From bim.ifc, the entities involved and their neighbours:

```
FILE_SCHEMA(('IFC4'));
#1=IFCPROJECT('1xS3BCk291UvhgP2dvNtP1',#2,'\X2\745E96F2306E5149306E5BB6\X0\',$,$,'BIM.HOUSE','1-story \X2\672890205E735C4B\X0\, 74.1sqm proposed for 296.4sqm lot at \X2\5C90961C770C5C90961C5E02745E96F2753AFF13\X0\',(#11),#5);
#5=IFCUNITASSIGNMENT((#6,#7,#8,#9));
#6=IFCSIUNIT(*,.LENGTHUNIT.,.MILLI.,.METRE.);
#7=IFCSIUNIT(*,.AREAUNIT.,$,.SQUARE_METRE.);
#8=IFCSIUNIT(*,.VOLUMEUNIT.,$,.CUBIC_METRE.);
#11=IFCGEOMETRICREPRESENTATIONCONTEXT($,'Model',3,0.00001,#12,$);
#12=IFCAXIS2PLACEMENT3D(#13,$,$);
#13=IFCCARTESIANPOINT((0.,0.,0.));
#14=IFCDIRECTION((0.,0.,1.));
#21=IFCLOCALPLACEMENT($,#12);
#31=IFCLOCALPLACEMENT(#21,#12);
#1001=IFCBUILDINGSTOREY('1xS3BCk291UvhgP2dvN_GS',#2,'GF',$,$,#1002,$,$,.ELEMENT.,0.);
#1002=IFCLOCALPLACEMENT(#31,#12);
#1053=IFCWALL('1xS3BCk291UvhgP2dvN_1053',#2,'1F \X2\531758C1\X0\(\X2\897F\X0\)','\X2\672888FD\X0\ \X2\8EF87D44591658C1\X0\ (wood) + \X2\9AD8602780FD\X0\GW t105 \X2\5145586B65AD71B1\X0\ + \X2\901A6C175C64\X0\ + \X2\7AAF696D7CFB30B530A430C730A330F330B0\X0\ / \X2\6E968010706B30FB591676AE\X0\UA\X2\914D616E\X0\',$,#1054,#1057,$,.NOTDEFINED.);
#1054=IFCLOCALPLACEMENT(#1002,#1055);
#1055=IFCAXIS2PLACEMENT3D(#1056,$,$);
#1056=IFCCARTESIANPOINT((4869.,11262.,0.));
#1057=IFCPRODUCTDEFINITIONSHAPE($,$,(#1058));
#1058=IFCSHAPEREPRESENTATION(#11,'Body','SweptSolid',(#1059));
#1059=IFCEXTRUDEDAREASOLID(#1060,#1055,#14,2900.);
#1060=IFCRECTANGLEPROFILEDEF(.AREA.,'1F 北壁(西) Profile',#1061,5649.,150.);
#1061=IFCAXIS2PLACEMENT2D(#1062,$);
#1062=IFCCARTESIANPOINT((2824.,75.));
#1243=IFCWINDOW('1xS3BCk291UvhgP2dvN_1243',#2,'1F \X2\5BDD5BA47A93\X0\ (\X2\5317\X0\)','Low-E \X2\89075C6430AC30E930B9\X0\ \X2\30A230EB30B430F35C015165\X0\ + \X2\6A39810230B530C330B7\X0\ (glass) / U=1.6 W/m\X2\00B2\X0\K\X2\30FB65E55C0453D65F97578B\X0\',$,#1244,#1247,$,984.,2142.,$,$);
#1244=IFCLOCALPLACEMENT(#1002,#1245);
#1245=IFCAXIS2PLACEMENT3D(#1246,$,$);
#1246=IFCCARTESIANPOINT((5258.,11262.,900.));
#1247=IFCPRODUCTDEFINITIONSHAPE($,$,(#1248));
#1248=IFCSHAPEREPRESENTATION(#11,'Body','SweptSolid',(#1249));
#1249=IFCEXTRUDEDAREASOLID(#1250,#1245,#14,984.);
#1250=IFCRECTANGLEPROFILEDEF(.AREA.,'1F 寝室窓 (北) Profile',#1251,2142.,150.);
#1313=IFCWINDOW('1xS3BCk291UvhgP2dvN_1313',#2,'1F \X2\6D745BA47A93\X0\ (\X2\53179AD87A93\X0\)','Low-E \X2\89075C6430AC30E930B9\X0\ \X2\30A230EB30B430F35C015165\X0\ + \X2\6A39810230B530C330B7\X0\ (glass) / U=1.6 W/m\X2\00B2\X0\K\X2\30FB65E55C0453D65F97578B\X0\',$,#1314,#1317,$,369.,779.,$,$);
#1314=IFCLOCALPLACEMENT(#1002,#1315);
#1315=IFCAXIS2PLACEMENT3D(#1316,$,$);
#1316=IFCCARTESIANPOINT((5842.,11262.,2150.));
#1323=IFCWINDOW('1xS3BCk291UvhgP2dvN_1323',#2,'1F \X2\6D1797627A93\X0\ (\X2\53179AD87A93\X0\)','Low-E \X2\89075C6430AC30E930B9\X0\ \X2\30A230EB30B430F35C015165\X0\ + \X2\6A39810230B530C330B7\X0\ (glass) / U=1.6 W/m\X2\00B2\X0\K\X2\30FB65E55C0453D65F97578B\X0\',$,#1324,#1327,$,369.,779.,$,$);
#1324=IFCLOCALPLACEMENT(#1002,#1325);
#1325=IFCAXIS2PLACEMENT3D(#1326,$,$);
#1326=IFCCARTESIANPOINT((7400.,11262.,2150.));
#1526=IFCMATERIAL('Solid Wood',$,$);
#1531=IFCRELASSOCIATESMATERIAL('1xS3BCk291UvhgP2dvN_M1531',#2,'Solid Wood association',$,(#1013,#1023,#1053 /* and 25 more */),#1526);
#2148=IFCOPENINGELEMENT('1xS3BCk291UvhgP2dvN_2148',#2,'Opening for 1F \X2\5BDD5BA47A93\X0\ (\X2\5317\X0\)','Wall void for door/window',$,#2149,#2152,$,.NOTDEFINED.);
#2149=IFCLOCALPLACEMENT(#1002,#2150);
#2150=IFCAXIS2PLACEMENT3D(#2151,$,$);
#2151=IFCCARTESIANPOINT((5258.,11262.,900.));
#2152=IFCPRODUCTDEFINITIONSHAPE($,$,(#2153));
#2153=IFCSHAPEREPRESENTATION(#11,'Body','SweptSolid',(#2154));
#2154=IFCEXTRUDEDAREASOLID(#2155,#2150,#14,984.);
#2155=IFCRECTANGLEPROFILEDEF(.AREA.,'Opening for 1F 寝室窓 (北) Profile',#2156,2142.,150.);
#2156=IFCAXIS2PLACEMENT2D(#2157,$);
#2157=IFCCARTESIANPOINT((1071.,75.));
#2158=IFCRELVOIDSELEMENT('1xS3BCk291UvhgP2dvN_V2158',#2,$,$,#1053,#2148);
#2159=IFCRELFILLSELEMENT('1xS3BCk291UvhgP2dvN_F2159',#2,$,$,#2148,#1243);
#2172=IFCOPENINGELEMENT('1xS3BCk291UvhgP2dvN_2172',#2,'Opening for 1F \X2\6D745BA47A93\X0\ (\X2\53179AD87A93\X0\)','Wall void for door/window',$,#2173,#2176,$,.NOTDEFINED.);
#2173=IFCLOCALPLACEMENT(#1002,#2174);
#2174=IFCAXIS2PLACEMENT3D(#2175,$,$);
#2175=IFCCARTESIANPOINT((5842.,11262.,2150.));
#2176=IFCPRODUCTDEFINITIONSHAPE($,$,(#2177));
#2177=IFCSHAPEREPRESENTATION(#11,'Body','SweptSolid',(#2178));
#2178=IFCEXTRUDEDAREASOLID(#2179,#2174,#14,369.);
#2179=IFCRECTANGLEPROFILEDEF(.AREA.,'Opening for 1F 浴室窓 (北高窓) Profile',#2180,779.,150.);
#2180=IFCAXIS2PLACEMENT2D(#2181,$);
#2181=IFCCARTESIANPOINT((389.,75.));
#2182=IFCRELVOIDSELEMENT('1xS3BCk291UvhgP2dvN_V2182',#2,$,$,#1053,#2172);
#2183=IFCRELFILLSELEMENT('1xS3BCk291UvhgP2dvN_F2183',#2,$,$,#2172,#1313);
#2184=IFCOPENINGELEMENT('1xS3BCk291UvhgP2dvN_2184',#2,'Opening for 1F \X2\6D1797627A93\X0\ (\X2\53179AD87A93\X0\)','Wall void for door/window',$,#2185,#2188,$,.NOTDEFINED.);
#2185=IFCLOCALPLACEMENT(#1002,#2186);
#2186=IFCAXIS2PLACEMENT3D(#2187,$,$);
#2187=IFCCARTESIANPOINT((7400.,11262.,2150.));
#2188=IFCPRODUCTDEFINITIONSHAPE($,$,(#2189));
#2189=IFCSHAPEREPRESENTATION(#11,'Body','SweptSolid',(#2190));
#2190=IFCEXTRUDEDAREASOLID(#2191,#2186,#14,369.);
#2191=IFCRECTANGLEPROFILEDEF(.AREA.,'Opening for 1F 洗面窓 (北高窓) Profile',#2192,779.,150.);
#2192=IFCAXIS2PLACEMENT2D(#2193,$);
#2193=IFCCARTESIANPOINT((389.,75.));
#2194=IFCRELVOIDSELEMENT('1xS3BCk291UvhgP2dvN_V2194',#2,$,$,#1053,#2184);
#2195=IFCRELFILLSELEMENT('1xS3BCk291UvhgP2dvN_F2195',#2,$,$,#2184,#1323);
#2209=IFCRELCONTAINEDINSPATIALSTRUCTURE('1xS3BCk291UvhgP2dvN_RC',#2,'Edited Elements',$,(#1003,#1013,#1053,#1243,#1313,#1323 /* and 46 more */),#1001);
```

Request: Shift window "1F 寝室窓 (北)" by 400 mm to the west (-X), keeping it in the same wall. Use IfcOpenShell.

```python
import ifcopenshell
import ifcopenshell.api.geometry
import ifcopenshell.util.placement
import ifcopenshell.util.unit

model = ifcopenshell.open("bim.ifc")
unit_scale = ifcopenshell.util.unit.calculate_unit_scale(model)

window = model.by_id(1243)
opening = window.FillsVoids[0].RelatingOpeningElement
wall = opening.VoidsElements[0].RelatingBuildingElement

wall_matrix = ifcopenshell.util.placement.get_local_placement(wall.ObjectPlacement)
shift = wall_matrix[:3, 0] * -0.4 / unit_scale
before = ifcopenshell.util.placement.get_local_placement(window.ObjectPlacement)[:3, 3].copy()

# The window is not placed relative to its opening, so move both.
for product in (opening, window):
    matrix = ifcopenshell.util.placement.get_local_placement(product.ObjectPlacement)
    matrix[:3, 3] += shift
    ifcopenshell.api.geometry.edit_object_placement(model, product=product, matrix=matrix, is_si=False)

after = ifcopenshell.util.placement.get_local_placement(window.ObjectPlacement)[:3, 3]
print("window moved by", (after - before).round(3) + 0.0)

model.write("bim_updated.ifc")
```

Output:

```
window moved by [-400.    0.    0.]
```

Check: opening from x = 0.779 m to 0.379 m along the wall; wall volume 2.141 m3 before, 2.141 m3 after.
